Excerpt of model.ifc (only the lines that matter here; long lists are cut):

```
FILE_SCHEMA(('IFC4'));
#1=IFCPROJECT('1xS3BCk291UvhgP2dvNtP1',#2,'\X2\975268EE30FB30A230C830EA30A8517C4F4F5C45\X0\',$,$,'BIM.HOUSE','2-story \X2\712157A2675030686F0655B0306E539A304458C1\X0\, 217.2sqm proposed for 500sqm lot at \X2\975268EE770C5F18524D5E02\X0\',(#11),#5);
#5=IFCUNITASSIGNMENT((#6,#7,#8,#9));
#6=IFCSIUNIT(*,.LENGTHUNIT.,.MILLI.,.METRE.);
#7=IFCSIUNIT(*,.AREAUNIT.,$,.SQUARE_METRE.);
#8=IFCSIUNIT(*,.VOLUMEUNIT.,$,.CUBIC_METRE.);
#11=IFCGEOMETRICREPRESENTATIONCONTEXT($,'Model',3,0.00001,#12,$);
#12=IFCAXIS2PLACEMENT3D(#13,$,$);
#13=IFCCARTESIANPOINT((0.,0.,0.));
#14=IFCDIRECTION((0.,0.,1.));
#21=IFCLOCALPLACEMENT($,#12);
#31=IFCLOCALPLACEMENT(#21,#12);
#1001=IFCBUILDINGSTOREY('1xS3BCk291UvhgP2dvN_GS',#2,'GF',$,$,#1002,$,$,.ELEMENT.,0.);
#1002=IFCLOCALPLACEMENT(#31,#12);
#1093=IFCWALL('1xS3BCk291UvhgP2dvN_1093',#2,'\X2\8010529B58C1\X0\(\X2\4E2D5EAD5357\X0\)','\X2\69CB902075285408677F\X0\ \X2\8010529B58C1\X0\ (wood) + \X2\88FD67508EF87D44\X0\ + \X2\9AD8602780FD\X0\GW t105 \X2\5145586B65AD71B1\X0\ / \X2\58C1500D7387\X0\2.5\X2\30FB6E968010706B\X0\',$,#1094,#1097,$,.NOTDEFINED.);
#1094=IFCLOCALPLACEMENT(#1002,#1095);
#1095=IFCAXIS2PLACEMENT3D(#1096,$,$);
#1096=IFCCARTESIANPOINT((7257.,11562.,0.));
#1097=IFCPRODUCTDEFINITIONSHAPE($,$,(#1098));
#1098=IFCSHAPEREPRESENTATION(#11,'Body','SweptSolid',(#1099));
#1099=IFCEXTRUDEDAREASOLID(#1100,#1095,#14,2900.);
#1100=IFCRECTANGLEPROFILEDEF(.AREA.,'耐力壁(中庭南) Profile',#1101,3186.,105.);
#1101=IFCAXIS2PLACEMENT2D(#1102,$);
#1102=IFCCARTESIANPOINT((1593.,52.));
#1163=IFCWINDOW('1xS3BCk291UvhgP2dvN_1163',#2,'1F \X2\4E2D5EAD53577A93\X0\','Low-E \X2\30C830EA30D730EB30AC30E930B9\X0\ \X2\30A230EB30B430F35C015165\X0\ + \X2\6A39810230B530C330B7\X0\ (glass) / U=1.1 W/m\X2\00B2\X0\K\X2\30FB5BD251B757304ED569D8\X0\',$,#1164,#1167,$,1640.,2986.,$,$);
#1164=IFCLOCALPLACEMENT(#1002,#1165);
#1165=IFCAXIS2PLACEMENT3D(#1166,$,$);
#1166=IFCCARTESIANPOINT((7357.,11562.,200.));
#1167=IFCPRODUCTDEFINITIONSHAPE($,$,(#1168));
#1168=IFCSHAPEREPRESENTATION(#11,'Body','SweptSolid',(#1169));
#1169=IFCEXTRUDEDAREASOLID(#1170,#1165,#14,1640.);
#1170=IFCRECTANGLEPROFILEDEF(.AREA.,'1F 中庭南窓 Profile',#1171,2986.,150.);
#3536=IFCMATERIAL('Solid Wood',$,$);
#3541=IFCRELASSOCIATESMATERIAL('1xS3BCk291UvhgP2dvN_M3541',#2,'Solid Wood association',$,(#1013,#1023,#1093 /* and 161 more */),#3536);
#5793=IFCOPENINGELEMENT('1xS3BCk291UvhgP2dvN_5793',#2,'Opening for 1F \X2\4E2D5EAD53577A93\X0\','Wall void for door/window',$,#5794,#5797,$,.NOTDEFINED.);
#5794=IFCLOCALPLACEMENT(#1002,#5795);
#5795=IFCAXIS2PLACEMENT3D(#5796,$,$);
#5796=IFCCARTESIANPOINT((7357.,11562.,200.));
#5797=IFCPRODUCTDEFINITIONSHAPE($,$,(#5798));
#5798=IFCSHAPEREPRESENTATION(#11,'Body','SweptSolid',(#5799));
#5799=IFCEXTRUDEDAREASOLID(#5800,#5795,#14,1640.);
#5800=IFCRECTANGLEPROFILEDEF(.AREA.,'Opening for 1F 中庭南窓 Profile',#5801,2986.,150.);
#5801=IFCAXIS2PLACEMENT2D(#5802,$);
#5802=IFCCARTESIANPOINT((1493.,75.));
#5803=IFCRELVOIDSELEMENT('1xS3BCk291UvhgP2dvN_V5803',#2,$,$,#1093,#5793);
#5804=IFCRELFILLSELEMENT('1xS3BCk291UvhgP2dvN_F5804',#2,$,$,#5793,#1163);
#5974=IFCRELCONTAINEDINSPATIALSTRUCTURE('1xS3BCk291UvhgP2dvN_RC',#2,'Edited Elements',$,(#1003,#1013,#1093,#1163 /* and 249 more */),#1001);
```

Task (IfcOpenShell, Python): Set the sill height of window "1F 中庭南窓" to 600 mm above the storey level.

```python
import numpy as np
import ifcopenshell
import ifcopenshell.api.geometry
import ifcopenshell.geom
import ifcopenshell.util.element
import ifcopenshell.util.placement
import ifcopenshell.util.shape
import ifcopenshell.util.unit

model = ifcopenshell.open("model.ifc")
unit_scale = ifcopenshell.util.unit.calculate_unit_scale(model)

window = model.by_guid("1xS3BCk291UvhgP2dvN_1163")
opening = window.FillsVoids[0].RelatingOpeningElement
storey = ifcopenshell.util.element.get_container(window, ifc_class="IfcBuildingStorey")
level = ifcopenshell.util.placement.get_local_placement(storey.ObjectPlacement)[2, 3]

# The opening's origin need not be at the sill, so measure its lowest point.
shape = ifcopenshell.geom.create_shape(ifcopenshell.geom.settings(), opening)
bottom = ifcopenshell.util.shape.get_shape_bottom_elevation(shape, shape.geometry) / unit_scale
dz = level + 0.6 / unit_scale - bottom

shift = np.array([0.0, 0.0, dz])
# The window is not placed relative to its opening, so move both.
for product in (opening, window):
    matrix = ifcopenshell.util.placement.get_local_placement(product.ObjectPlacement)
    matrix[:3, 3] += shift
    ifcopenshell.api.geometry.edit_object_placement(model, product=product, matrix=matrix, is_si=False)

print(f"moved by {dz * unit_scale:+.3f} m")

model.write("model_edited.ifc")
```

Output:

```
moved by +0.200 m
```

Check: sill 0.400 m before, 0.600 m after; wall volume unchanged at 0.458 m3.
